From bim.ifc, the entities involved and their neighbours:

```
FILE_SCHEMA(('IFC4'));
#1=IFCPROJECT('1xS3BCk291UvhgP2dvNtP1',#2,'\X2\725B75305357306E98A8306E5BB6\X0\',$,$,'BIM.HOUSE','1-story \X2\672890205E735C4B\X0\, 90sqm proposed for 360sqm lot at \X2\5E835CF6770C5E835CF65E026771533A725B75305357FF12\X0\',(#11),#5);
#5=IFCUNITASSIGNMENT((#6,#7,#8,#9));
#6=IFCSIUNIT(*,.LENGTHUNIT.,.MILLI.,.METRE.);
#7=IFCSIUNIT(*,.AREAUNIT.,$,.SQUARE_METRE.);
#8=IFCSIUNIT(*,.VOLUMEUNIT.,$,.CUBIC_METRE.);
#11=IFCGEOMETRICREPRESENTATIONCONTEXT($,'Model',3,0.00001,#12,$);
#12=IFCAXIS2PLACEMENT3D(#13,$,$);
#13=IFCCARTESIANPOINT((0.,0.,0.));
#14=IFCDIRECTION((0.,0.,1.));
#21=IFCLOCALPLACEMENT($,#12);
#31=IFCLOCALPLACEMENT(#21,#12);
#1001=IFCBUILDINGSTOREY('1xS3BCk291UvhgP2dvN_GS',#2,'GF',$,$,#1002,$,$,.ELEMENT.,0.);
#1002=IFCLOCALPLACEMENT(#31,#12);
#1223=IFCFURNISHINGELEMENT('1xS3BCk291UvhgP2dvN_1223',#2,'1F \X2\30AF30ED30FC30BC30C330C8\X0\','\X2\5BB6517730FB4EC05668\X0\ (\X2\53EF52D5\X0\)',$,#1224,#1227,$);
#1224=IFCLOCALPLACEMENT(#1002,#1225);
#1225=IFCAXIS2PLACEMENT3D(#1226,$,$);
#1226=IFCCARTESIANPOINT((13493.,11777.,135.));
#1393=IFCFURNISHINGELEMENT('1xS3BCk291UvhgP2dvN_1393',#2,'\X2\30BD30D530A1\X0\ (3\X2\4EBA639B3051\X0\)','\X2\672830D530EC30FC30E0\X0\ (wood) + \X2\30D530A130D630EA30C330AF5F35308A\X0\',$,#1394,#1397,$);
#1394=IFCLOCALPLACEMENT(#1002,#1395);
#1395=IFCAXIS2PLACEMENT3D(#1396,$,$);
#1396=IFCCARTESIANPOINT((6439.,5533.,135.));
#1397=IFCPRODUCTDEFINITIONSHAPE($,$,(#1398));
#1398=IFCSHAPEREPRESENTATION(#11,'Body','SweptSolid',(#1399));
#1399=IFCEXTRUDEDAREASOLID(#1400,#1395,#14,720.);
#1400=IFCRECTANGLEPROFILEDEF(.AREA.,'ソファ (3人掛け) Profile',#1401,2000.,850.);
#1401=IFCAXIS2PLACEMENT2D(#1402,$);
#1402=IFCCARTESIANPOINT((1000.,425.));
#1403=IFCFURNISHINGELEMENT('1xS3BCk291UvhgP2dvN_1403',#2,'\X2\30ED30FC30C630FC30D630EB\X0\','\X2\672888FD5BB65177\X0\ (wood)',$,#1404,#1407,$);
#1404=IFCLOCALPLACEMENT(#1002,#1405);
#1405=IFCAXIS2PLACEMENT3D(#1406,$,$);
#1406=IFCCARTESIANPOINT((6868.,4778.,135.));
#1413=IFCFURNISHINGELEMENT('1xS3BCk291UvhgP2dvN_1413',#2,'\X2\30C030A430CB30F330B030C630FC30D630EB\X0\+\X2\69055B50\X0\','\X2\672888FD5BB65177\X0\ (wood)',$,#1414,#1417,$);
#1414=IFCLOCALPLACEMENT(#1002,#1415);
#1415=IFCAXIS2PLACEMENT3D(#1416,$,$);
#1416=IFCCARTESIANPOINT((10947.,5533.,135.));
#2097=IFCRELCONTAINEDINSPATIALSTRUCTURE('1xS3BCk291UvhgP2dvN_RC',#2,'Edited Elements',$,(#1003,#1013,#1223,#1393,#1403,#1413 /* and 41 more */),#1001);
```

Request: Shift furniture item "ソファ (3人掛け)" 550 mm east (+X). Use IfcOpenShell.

```python
import ifcopenshell
import ifcopenshell.api.geometry
import ifcopenshell.util.placement

model = ifcopenshell.open("bim.ifc")

item = model.by_id(1393)
matrix = ifcopenshell.util.placement.get_local_placement(item.ObjectPlacement)
matrix[0, 3] += 550.0
ifcopenshell.api.geometry.edit_object_placement(model, product=item, matrix=matrix, is_si=False)

print(ifcopenshell.util.placement.get_local_placement(item.ObjectPlacement).round(3) + 0.0)

model.write("bim_rev.ifc")
```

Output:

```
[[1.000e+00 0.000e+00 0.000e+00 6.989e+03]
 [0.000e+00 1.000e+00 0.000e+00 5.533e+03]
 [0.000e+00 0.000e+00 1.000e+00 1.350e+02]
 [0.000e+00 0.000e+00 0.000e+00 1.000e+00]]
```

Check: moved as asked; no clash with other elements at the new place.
